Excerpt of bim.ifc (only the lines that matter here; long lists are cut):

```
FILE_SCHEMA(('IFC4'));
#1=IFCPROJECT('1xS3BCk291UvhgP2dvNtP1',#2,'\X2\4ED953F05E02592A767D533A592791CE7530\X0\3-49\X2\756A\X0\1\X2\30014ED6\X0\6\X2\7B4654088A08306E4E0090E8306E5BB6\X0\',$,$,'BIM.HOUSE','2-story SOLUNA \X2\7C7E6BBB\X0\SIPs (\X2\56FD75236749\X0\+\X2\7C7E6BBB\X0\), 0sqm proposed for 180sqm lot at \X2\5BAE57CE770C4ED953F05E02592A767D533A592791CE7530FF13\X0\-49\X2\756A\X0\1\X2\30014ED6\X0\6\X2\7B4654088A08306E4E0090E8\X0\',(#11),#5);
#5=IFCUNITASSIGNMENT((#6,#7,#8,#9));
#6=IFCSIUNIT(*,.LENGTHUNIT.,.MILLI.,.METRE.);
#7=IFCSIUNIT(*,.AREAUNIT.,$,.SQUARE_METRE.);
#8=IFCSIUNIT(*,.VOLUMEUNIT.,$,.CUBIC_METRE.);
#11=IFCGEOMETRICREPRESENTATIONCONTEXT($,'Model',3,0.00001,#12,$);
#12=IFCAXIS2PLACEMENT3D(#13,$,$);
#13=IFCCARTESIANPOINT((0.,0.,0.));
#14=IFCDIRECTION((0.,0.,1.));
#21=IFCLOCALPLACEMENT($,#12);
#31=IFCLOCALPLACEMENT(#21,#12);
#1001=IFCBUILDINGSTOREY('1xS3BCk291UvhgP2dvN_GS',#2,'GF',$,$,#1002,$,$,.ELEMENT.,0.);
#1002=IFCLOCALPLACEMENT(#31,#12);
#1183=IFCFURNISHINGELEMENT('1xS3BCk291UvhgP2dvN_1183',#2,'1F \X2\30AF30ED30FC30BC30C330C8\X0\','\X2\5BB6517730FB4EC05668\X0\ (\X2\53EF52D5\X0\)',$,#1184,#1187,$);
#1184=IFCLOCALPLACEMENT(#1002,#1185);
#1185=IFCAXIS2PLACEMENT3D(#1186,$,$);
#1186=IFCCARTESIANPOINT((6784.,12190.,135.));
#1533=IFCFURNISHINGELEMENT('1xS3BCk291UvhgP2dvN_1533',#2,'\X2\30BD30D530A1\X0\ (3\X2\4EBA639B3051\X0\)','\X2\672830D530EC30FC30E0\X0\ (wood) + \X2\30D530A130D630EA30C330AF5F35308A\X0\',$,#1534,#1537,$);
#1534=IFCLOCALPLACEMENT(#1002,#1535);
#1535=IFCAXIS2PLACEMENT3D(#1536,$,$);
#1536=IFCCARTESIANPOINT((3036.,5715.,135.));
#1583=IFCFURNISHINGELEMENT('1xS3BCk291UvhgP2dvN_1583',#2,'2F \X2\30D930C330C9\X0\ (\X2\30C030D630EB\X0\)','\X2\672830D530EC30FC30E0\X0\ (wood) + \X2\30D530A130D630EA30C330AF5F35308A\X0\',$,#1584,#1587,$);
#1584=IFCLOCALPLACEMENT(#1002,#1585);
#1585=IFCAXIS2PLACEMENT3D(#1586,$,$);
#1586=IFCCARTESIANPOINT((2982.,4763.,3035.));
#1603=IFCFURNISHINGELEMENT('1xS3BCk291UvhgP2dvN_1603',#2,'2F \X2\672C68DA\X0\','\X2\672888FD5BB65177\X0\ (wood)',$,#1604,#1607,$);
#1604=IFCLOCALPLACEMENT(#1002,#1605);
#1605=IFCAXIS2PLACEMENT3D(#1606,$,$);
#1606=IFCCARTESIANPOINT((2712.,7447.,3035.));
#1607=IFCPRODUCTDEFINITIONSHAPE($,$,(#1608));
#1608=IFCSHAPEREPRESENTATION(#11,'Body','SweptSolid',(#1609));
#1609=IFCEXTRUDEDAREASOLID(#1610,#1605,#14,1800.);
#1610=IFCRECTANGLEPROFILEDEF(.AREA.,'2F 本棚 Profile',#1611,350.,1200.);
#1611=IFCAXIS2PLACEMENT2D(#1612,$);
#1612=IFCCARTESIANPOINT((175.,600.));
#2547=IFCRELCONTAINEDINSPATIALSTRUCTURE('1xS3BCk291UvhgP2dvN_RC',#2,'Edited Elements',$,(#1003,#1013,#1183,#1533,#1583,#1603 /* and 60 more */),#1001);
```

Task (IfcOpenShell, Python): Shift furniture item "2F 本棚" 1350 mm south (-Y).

```python
import ifcopenshell
import ifcopenshell.api.geometry
import ifcopenshell.util.placement
import ifcopenshell.util.unit

model = ifcopenshell.open("bim.ifc")
unit_scale = ifcopenshell.util.unit.calculate_unit_scale(model)

item = model.by_guid("1xS3BCk291UvhgP2dvN_1603")
matrix = ifcopenshell.util.placement.get_local_placement(item.ObjectPlacement)
matrix[1, 3] -= 1.35 / unit_scale
ifcopenshell.api.geometry.edit_object_placement(model, product=item, matrix=matrix, is_si=False)

print(ifcopenshell.util.placement.get_local_placement(item.ObjectPlacement).round(3) + 0.0)

model.write("bim_updated.ifc")
```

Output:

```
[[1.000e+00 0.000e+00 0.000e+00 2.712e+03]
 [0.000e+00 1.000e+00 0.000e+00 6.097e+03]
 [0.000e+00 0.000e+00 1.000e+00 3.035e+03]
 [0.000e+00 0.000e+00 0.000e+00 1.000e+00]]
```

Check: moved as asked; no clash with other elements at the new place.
